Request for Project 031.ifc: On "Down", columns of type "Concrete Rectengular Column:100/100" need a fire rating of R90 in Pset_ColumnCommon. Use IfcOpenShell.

First a look at what the model holds.

```python
import ifcopenshell
import ifcopenshell.util.element

model = ifcopenshell.open("Project 031.ifc")
print(model.schema)
storey = next(s for s in model.by_type("IfcBuildingStorey") if s.Name == "Down")
columns = [e for e in ifcopenshell.util.element.get_decomposition(storey) if e.is_a("IfcColumn")]
seen = {}
for e in columns:
    element_type = ifcopenshell.util.element.get_type(e)
    key = (element_type.Name if element_type != e and element_type else None, ifcopenshell.util.element.get_pset(e, "Pset_ColumnCommon", "FireRating"))
    seen[key] = seen.get(key, 0) + 1
for (name, value), count in sorted(seen.items(), key=str):
    print(count, "x", name, "|", value)
```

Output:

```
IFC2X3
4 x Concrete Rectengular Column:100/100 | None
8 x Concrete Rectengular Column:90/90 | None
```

```python
import ifcopenshell
import ifcopenshell.api.pset
import ifcopenshell.util.element

model = ifcopenshell.open("Project 031.ifc")

storey = next(s for s in model.by_type("IfcBuildingStorey") if s.Name == "Down")
columns = [e for e in ifcopenshell.util.element.get_decomposition(storey) if e.is_a("IfcColumn")]

count = 0
for e in columns:
    element_type = ifcopenshell.util.element.get_type(e)
    if element_type in (None, e) or element_type.Name != "Concrete Rectengular Column:100/100":
        continue
    # add_pset returns the element's existing set when there is one.
    pset = ifcopenshell.api.pset.add_pset(model, product=e, name="Pset_ColumnCommon")
    ifcopenshell.api.pset.edit_pset(model, pset=pset, properties={"FireRating": "R90"})
    count += 1

print(count, "columns updated")

model.write("Project 031-out.ifc")
```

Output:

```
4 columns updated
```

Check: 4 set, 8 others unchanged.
